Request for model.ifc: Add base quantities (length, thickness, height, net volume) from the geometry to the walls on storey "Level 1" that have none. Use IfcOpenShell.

First a look at what the model holds.

```python
import ifcopenshell
import ifcopenshell.util.element
import ifcopenshell.util.unit

model = ifcopenshell.open("model.ifc")
print(model.schema)
for unit_type in ("LENGTHUNIT", "AREAUNIT", "VOLUMEUNIT"):
    print(unit_type, ifcopenshell.util.unit.calculate_unit_scale(model, unit_type))
storey = next(s for s in model.by_type("IfcBuildingStorey") if s.Name == "Level 1")
walls = [e for e in ifcopenshell.util.element.get_decomposition(storey) if e.is_a("IfcWall")]
for e in sorted(walls, key=lambda e: e.id()):
    print(e.id(), e.is_a(), e.Name, list(ifcopenshell.util.element.get_psets(e, qtos_only=True)), sep=" | ")
```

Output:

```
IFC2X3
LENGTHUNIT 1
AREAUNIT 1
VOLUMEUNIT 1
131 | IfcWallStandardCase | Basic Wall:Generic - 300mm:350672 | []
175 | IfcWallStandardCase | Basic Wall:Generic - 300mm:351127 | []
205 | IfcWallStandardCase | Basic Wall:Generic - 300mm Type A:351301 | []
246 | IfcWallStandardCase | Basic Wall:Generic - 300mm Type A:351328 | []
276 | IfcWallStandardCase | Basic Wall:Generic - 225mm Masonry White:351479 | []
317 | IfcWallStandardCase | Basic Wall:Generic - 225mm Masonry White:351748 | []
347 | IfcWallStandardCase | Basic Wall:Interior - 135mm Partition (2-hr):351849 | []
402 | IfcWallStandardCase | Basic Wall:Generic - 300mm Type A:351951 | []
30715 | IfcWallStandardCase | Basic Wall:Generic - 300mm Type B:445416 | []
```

```python
import ifcopenshell
import ifcopenshell.api.pset
import ifcopenshell.geom
import ifcopenshell.util.element
import ifcopenshell.util.shape
import ifcopenshell.util.unit

model = ifcopenshell.open("model.ifc")
unit_scale = ifcopenshell.util.unit.calculate_unit_scale(model)
volume_scale = ifcopenshell.util.unit.calculate_unit_scale(model, "VOLUMEUNIT")
settings = ifcopenshell.geom.settings()

storey = next(s for s in model.by_type("IfcBuildingStorey") if s.Name == "Level 1")
walls = [e for e in ifcopenshell.util.element.get_decomposition(storey) if e.is_a("IfcWall")]

for e in sorted(walls, key=lambda e: e.id()):
    if ifcopenshell.util.element.get_psets(e, qtos_only=True, should_inherit=False):
        continue
    # Geometry comes back in metres, in the element's own axes.
    shape = ifcopenshell.geom.create_shape(settings, e)
    values = {
        "Length": ifcopenshell.util.shape.get_x(shape.geometry) / unit_scale,
        "Width": ifcopenshell.util.shape.get_y(shape.geometry) / unit_scale,
        "Height": ifcopenshell.util.shape.get_z(shape.geometry) / unit_scale,
        "NetVolume": ifcopenshell.util.shape.get_volume(shape.geometry) / volume_scale,
    }
    qto = ifcopenshell.api.pset.add_qto(model, product=e, name="BaseQuantities")
    ifcopenshell.api.pset.edit_qto(model, qto=qto, properties=values)
    print(e.id(), {k: round(v, 3) for k, v in values.items()})

model.write("model_rev.ifc")
```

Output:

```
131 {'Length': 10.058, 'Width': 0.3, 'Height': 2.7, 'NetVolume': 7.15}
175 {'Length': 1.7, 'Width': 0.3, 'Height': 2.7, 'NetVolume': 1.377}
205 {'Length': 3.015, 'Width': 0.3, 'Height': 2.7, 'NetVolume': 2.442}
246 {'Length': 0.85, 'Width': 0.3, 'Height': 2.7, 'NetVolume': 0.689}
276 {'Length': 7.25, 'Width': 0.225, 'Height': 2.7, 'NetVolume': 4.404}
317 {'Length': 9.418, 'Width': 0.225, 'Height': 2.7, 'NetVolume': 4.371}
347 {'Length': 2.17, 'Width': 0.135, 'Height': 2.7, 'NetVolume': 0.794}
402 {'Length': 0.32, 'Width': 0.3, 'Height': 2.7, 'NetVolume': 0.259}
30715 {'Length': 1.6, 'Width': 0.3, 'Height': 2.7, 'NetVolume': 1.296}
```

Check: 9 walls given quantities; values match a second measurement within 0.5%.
